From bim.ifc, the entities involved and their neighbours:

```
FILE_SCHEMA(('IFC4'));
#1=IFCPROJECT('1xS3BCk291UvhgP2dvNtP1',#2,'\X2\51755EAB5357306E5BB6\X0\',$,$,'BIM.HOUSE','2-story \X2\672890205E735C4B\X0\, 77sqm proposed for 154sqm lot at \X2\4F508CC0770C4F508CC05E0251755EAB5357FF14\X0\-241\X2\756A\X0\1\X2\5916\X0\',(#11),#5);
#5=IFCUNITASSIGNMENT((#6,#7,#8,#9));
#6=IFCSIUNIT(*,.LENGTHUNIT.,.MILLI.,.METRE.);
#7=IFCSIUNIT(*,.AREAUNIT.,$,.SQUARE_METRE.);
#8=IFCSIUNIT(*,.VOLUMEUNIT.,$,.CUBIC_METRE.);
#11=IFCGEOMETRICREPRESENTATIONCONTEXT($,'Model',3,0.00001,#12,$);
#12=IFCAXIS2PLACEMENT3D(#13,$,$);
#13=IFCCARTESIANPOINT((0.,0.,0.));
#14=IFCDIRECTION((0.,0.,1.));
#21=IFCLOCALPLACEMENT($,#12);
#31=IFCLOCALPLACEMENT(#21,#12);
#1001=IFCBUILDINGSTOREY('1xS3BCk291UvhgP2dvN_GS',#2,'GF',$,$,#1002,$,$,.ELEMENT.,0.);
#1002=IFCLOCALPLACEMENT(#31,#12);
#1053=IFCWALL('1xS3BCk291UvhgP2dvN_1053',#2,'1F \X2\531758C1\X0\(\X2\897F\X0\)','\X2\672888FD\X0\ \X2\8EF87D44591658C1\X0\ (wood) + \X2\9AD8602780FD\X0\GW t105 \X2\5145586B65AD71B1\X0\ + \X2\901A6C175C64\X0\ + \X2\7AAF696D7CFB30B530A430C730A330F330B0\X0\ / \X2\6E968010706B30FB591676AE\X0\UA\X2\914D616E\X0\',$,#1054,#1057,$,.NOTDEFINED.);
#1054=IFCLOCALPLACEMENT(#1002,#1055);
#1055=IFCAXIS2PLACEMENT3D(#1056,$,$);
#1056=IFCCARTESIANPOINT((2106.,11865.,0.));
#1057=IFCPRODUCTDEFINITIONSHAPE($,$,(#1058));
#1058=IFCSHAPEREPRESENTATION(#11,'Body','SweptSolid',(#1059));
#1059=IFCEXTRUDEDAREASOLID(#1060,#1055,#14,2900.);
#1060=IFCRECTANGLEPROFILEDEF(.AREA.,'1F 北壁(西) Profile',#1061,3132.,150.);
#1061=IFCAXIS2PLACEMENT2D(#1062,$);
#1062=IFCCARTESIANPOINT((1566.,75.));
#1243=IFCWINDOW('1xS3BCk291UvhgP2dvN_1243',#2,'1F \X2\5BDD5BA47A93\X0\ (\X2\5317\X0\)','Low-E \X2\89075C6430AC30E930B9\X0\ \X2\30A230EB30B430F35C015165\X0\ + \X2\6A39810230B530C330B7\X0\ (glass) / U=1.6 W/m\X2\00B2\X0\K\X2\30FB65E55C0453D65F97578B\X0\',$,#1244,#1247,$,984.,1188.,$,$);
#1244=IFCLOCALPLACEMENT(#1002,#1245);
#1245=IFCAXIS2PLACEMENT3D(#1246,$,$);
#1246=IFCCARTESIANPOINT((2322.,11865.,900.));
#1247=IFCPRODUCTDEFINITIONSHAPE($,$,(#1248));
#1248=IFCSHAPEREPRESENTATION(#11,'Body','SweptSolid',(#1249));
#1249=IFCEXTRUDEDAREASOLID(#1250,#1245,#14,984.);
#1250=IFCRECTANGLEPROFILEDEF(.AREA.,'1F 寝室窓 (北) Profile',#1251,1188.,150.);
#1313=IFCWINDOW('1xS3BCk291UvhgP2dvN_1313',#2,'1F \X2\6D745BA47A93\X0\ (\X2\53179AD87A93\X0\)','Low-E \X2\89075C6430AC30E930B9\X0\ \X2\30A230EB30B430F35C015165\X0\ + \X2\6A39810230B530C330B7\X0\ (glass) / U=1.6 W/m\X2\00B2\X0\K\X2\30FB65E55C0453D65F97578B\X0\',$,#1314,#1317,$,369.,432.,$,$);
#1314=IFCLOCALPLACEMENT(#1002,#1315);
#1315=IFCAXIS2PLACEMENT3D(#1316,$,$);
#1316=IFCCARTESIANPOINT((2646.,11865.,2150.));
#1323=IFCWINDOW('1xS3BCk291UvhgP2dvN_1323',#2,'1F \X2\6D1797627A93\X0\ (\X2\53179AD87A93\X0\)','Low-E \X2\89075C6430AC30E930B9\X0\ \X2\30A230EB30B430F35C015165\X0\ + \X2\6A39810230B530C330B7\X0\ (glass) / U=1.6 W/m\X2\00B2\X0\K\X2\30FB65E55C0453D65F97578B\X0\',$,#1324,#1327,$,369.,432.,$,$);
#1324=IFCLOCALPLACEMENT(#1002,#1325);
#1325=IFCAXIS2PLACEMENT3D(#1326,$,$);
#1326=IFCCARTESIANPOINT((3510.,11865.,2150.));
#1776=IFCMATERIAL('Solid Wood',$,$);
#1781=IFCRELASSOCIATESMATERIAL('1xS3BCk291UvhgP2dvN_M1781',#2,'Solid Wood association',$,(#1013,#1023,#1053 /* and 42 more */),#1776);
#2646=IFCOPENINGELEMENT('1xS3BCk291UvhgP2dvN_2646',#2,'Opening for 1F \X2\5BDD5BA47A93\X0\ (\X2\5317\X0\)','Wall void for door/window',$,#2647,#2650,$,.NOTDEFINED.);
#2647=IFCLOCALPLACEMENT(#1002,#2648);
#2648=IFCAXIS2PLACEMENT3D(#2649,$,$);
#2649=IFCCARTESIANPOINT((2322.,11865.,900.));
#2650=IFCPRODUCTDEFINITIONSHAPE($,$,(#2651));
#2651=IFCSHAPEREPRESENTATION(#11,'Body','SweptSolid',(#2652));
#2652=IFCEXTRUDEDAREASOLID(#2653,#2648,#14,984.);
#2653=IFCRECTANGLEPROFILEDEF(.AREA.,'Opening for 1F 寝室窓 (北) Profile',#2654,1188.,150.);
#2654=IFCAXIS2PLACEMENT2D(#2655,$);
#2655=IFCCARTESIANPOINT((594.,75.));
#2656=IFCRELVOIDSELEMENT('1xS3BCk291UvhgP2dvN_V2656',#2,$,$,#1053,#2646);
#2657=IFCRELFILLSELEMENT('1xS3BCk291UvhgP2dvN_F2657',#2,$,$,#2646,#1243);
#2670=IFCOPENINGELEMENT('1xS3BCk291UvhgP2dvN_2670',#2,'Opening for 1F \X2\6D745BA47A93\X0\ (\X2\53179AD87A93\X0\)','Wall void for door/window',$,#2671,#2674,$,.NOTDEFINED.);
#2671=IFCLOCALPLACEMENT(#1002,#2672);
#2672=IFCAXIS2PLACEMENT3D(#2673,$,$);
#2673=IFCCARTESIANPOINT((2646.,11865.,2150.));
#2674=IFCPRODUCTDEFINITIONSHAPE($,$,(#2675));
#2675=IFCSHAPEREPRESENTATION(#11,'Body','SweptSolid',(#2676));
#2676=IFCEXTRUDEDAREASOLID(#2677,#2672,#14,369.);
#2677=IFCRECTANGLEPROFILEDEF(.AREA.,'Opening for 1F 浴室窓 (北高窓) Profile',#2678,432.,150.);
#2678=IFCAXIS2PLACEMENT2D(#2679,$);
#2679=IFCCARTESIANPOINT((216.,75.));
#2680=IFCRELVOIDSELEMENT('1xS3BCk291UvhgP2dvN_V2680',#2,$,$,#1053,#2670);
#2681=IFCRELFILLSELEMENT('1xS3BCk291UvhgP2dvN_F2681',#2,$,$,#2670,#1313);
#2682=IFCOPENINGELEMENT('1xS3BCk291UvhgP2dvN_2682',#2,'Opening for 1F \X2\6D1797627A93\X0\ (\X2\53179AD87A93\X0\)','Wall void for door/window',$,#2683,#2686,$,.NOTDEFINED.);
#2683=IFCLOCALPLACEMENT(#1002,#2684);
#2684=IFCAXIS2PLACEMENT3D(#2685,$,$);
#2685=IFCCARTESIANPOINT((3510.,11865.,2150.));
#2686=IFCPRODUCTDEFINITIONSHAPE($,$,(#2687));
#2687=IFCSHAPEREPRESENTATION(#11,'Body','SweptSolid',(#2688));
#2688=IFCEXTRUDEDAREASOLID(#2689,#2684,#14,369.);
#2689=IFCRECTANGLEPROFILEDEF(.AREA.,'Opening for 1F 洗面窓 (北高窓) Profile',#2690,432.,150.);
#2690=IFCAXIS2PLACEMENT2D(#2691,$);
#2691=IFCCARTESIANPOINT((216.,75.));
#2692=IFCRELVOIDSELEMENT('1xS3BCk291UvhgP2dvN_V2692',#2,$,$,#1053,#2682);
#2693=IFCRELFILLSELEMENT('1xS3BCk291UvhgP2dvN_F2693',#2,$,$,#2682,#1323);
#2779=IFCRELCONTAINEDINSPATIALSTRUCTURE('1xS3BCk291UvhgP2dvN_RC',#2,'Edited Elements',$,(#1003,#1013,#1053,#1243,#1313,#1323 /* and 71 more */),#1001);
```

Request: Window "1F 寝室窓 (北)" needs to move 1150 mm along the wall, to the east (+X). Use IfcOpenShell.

```python
import ifcopenshell
import ifcopenshell.api.geometry
import ifcopenshell.util.placement
import ifcopenshell.util.unit

model = ifcopenshell.open("bim.ifc")
unit_scale = ifcopenshell.util.unit.calculate_unit_scale(model)

window = model.by_guid("1xS3BCk291UvhgP2dvN_1243")
opening = window.FillsVoids[0].RelatingOpeningElement
wall = opening.VoidsElements[0].RelatingBuildingElement

wall_matrix = ifcopenshell.util.placement.get_local_placement(wall.ObjectPlacement)
shift = wall_matrix[:3, 0] * 1.15 / unit_scale
before = ifcopenshell.util.placement.get_local_placement(window.ObjectPlacement)[:3, 3].copy()

# The window is not placed relative to its opening, so move both.
for product in (opening, window):
    matrix = ifcopenshell.util.placement.get_local_placement(product.ObjectPlacement)
    matrix[:3, 3] += shift
    ifcopenshell.api.geometry.edit_object_placement(model, product=product, matrix=matrix, is_si=False)

after = ifcopenshell.util.placement.get_local_placement(window.ObjectPlacement)[:3, 3]
print("window moved by", (after - before).round(3) + 0.0)

model.write("bim_edited.ifc")
```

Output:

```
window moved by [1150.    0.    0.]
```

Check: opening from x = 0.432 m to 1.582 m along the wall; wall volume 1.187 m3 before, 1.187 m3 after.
